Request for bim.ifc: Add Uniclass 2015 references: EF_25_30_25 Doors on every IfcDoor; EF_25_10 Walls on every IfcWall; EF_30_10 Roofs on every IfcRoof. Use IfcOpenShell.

First a look at what the model holds.

```python
import ifcopenshell

model = ifcopenshell.open("bim.ifc")
print(model.schema)
print("classifications:", [c.Name for c in model.by_type("IfcClassification")])
for ifc_class in ("IfcDoor", "IfcRoof", "IfcStair", "IfcWall", "IfcWindow"):
    print(ifc_class, len(model.by_type(ifc_class)))
```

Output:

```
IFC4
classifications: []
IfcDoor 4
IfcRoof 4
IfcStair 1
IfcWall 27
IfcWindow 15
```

```python
import ifcopenshell
import ifcopenshell.api.classification

model = ifcopenshell.open("bim.ifc")

system = ifcopenshell.api.classification.add_classification(model, classification="Uniclass 2015")

codes = {
    "IfcDoor": ("EF_25_30_25", "Doors"),
    "IfcWall": ("EF_25_10", "Walls"),
    "IfcRoof": ("EF_30_10", "Roofs"),
}
for ifc_class, (code, name) in codes.items():
    products = model.by_type(ifc_class)
    ifcopenshell.api.classification.add_reference(
        model, products=products, classification=system, identification=code, name=name
    )
    print(code, len(products))

model.write("bim-out.ifc")
```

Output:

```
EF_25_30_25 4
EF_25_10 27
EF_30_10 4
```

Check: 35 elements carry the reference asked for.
